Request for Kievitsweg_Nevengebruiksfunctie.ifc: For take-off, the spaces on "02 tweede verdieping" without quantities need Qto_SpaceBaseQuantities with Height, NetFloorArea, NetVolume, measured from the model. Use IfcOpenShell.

First a look at what the model holds.

```python
import ifcopenshell
import ifcopenshell.util.element
import ifcopenshell.util.unit

model = ifcopenshell.open("Kievitsweg_Nevengebruiksfunctie.ifc")
print(model.schema)
for unit_type in ("LENGTHUNIT", "AREAUNIT", "VOLUMEUNIT"):
    print(unit_type, ifcopenshell.util.unit.calculate_unit_scale(model, unit_type))
storey = next(s for s in model.by_type("IfcBuildingStorey") if s.Name == "02 tweede verdieping")
spaces = [e for e in ifcopenshell.util.element.get_decomposition(storey) if e.is_a("IfcSpace")]
for e in sorted(spaces, key=lambda e: e.id()):
    print(e.id(), e.is_a(), e.Name, list(ifcopenshell.util.element.get_psets(e, qtos_only=True)), sep=" | ")
```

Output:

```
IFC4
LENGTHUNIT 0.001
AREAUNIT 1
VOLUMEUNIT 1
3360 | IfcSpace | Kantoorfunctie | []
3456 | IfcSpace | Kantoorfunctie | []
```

```python
import ifcopenshell
import ifcopenshell.api.pset
import ifcopenshell.geom
import ifcopenshell.util.element
import ifcopenshell.util.shape
import ifcopenshell.util.unit

model = ifcopenshell.open("Kievitsweg_Nevengebruiksfunctie.ifc")
unit_scale = ifcopenshell.util.unit.calculate_unit_scale(model)
area_scale = ifcopenshell.util.unit.calculate_unit_scale(model, "AREAUNIT")
volume_scale = ifcopenshell.util.unit.calculate_unit_scale(model, "VOLUMEUNIT")
settings = ifcopenshell.geom.settings()

storey = next(s for s in model.by_type("IfcBuildingStorey") if s.Name == "02 tweede verdieping")
spaces = [e for e in ifcopenshell.util.element.get_decomposition(storey) if e.is_a("IfcSpace")]

for e in sorted(spaces, key=lambda e: e.id()):
    if ifcopenshell.util.element.get_psets(e, qtos_only=True, should_inherit=False):
        continue
    # Geometry comes back in metres, in the element's own axes.
    shape = ifcopenshell.geom.create_shape(settings, e)
    values = {
        "Height": ifcopenshell.util.shape.get_z(shape.geometry) / unit_scale,
        "NetFloorArea": ifcopenshell.util.shape.get_footprint_area(shape.geometry) / area_scale,
        "NetVolume": ifcopenshell.util.shape.get_volume(shape.geometry) / volume_scale,
    }
    qto = ifcopenshell.api.pset.add_qto(model, product=e, name="Qto_SpaceBaseQuantities")
    ifcopenshell.api.pset.edit_qto(model, qto=qto, properties=values)
    print(e.id(), {k: round(v, 3) for k, v in values.items()})

model.write("Kievitsweg_Nevengebruiksfunctie_edited.ifc")
```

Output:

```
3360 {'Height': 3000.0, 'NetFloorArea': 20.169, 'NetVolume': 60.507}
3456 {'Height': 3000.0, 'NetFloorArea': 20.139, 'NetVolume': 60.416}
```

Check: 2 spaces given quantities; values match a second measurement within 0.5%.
